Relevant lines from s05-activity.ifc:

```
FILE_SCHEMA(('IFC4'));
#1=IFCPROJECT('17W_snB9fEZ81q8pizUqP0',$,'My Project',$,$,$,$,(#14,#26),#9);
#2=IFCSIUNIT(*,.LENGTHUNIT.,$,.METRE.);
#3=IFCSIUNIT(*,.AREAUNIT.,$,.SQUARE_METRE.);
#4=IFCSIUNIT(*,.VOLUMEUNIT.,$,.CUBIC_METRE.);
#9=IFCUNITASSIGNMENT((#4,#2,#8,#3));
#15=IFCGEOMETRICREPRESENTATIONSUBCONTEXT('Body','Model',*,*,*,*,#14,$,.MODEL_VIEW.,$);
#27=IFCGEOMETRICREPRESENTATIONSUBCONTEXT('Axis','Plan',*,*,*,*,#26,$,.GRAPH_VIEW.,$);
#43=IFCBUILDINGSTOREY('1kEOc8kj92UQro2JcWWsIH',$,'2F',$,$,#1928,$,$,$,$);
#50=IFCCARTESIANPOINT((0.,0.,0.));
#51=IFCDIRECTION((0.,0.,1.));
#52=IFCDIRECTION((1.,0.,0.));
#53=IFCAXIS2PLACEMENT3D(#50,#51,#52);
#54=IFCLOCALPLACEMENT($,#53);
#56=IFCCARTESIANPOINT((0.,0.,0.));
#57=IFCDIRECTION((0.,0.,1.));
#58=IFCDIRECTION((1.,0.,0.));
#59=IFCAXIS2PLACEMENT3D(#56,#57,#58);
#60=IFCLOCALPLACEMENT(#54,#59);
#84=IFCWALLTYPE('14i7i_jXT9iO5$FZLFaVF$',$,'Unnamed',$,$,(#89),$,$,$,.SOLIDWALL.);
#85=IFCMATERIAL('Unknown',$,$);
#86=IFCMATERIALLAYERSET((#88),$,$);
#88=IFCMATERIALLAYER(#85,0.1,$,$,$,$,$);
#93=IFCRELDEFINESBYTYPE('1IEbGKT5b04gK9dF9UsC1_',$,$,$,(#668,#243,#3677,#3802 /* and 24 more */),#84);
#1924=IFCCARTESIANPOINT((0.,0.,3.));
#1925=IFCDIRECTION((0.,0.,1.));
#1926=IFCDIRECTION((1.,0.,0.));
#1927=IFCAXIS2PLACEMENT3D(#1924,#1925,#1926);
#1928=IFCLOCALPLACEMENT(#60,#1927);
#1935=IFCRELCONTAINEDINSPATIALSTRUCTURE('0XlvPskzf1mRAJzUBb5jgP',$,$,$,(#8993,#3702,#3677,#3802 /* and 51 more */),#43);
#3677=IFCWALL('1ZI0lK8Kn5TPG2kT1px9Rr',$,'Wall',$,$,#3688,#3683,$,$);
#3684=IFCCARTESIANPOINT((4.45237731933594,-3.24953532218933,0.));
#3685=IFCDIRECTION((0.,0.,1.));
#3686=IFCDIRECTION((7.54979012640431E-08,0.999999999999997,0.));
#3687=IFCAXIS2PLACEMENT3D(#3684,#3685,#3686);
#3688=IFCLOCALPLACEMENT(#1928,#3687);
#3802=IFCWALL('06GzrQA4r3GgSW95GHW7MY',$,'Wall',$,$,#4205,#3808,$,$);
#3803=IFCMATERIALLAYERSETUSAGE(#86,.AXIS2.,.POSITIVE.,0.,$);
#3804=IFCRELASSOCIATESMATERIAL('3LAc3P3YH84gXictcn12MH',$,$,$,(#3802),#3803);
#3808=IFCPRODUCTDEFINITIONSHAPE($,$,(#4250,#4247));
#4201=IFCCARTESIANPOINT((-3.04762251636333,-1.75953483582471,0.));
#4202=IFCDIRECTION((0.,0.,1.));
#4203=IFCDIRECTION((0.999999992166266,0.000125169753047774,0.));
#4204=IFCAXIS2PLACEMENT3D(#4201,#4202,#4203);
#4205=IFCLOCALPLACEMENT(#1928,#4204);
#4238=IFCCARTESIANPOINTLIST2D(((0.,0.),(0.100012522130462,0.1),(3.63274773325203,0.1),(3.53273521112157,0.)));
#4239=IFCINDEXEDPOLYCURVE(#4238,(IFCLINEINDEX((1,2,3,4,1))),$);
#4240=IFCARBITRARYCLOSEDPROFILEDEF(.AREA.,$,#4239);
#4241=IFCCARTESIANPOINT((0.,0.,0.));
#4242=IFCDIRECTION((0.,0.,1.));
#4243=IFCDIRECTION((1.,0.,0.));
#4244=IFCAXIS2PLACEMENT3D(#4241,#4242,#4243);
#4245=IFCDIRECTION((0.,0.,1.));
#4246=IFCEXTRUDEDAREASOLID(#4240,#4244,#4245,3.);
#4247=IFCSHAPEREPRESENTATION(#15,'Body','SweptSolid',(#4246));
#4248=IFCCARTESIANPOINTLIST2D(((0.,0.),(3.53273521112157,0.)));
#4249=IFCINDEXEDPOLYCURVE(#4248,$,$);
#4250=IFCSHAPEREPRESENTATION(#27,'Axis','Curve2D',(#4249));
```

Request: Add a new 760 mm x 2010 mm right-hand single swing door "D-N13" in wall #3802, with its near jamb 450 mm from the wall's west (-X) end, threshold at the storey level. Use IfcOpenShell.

```python
import numpy as np
import ifcopenshell
import ifcopenshell.api.feature
import ifcopenshell.api.geometry
import ifcopenshell.api.root
import ifcopenshell.api.spatial
import ifcopenshell.geom
import ifcopenshell.util.element
import ifcopenshell.util.placement
import ifcopenshell.util.representation
import ifcopenshell.util.shape
import ifcopenshell.util.unit

model = ifcopenshell.open("s05-activity.ifc")
unit_scale = ifcopenshell.util.unit.calculate_unit_scale(model)
settings = ifcopenshell.geom.settings()


def volume(element):
    """Net volume in cubic metres, openings subtracted."""
    shape = ifcopenshell.geom.create_shape(settings, element)
    return ifcopenshell.util.shape.get_volume(shape.geometry)


wall = model.by_guid("06GzrQA4r3GgSW95GHW7MY")
storey = ifcopenshell.util.element.get_container(wall, ifc_class="IfcBuildingStorey")
context = ifcopenshell.util.representation.get_context(model, "Model", "Body", "MODEL_VIEW")
before = volume(wall)

width, height, from_end, sill = 0.76, 2.01, 0.45, 0.0  # metres

# The wall runs along its own X axis, and the end named is its -X end.
wall_shape = ifcopenshell.geom.create_shape(settings, wall)
x, y, z = ifcopenshell.util.shape.get_vertices(wall_shape.geometry).T
start = x.min() + from_end
face, thickness = float(y.min()), float(y.max() - y.min())
wall_matrix = ifcopenshell.util.placement.get_local_placement(wall.ObjectPlacement)
level = ifcopenshell.util.placement.get_local_placement(storey.ObjectPlacement)[2, 3]


def in_wall(x, y):
    """Placement at x, y metres in the wall's axes, at sill height."""
    matrix = wall_matrix.copy()
    matrix[:, 3] = wall_matrix @ np.array([x / unit_scale, y / unit_scale, 0.0, 1.0])
    matrix[2, 3] = level + sill / unit_scale
    return matrix


# Opening: a box that overshoots both wall faces by 50 mm.
opening = ifcopenshell.api.root.create_entity(model, ifc_class="IfcOpeningElement", predefined_type="OPENING")
box = ifcopenshell.api.geometry.add_wall_representation(
    model, context=context, length=width, height=height, thickness=thickness + 0.1
)
ifcopenshell.api.geometry.assign_representation(model, product=opening, representation=box)
ifcopenshell.api.geometry.edit_object_placement(model, product=opening, matrix=in_wall(start, face - 0.05), is_si=False)
ifcopenshell.api.feature.add_feature(model, feature=opening, element=wall)

door = ifcopenshell.api.root.create_entity(model, ifc_class="IfcDoor", name="D-N13", predefined_type="DOOR")
door.OverallWidth, door.OverallHeight = width / unit_scale, height / unit_scale
door.OperationType = "SINGLE_SWING_RIGHT"
body = ifcopenshell.api.geometry.add_door_representation(
    model,
    context=context,
    overall_width=door.OverallWidth,
    overall_height=door.OverallHeight,
    operation_type="SINGLE_SWING_RIGHT",
    lining_properties={"LiningDepth": thickness / unit_scale, "ThresholdDepth": thickness / unit_scale},
)
ifcopenshell.api.geometry.assign_representation(model, product=door, representation=body)
ifcopenshell.api.spatial.assign_container(model, products=[door], relating_structure=storey)
ifcopenshell.api.feature.add_filling(model, opening=opening, element=door)

# The lining spans the wall, so the door starts at the wall face.
ifcopenshell.api.geometry.edit_object_placement(model, product=door, matrix=in_wall(start, face), is_si=False)

after = volume(wall)

print(f"wall volume {before:.3f} -> {after:.3f} m3")

model.write("s05-activity-out.ifc")
```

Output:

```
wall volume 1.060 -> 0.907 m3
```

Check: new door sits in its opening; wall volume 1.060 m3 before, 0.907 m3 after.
